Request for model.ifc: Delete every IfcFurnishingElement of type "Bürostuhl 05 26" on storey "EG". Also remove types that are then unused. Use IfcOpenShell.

First a look at what the model holds.

```python
import ifcopenshell
import ifcopenshell.util.element

model = ifcopenshell.open("model.ifc")
print(model.schema)
storey = next(s for s in model.by_type("IfcBuildingStorey") if s.Name == "EG")
furniture = [e for e in ifcopenshell.util.element.get_decomposition(storey) if e.is_a("IfcFurnishingElement")]
seen = {}
for e in furniture:
    element_type = ifcopenshell.util.element.get_type(e)
    name = element_type.Name if element_type not in (None, e) else None
    seen[name] = seen.get(name, 0) + 1
for name, count in sorted(seen.items(), key=str):
    print(count, "x", name)
```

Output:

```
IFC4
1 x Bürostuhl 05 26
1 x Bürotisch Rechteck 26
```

```python
import ifcopenshell
import ifcopenshell.api.root
import ifcopenshell.util.element

model = ifcopenshell.open("model.ifc")

storey = next(s for s in model.by_type("IfcBuildingStorey") if s.Name == "EG")
furniture = [e for e in ifcopenshell.util.element.get_decomposition(storey) if e.is_a("IfcFurnishingElement")]
targets = [e for e in furniture if (t := ifcopenshell.util.element.get_type(e)) not in (None, e) and t.Name == "Bürostuhl 05 26"]
types = {ifcopenshell.util.element.get_type(e) for e in targets} - {None, *targets}

for e in targets:
    ifcopenshell.api.root.remove_product(model, product=e)
print(len(targets), "removed")

unused = [t for t in types if not ifcopenshell.util.element.get_types(t)]
for t in unused:
    ifcopenshell.api.root.remove_product(model, product=t)
print(len(unused), "unused types removed")

model.write("model-out.ifc")
```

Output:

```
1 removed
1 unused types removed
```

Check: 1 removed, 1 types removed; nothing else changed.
